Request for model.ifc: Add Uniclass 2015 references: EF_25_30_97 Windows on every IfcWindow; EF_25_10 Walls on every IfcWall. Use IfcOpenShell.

First a look at what the model holds.

```python
import ifcopenshell

model = ifcopenshell.open("model.ifc")
print(model.schema)
print("classifications:", [c.Name for c in model.by_type("IfcClassification")])
for ifc_class in ("IfcDoor", "IfcRoof", "IfcStair", "IfcWall", "IfcWindow"):
    print(ifc_class, len(model.by_type(ifc_class)))
```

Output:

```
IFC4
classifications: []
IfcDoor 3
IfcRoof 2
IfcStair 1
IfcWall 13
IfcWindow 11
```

```python
import ifcopenshell
import ifcopenshell.api.classification

model = ifcopenshell.open("model.ifc")

system = ifcopenshell.api.classification.add_classification(model, classification="Uniclass 2015")

codes = {
    "IfcWindow": ("EF_25_30_97", "Windows"),
    "IfcWall": ("EF_25_10", "Walls"),
}
for ifc_class, (code, name) in codes.items():
    products = model.by_type(ifc_class)
    ifcopenshell.api.classification.add_reference(
        model, products=products, classification=system, identification=code, name=name
    )
    print(code, len(products))

model.write("model_rev.ifc")
```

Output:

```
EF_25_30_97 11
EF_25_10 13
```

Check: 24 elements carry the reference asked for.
